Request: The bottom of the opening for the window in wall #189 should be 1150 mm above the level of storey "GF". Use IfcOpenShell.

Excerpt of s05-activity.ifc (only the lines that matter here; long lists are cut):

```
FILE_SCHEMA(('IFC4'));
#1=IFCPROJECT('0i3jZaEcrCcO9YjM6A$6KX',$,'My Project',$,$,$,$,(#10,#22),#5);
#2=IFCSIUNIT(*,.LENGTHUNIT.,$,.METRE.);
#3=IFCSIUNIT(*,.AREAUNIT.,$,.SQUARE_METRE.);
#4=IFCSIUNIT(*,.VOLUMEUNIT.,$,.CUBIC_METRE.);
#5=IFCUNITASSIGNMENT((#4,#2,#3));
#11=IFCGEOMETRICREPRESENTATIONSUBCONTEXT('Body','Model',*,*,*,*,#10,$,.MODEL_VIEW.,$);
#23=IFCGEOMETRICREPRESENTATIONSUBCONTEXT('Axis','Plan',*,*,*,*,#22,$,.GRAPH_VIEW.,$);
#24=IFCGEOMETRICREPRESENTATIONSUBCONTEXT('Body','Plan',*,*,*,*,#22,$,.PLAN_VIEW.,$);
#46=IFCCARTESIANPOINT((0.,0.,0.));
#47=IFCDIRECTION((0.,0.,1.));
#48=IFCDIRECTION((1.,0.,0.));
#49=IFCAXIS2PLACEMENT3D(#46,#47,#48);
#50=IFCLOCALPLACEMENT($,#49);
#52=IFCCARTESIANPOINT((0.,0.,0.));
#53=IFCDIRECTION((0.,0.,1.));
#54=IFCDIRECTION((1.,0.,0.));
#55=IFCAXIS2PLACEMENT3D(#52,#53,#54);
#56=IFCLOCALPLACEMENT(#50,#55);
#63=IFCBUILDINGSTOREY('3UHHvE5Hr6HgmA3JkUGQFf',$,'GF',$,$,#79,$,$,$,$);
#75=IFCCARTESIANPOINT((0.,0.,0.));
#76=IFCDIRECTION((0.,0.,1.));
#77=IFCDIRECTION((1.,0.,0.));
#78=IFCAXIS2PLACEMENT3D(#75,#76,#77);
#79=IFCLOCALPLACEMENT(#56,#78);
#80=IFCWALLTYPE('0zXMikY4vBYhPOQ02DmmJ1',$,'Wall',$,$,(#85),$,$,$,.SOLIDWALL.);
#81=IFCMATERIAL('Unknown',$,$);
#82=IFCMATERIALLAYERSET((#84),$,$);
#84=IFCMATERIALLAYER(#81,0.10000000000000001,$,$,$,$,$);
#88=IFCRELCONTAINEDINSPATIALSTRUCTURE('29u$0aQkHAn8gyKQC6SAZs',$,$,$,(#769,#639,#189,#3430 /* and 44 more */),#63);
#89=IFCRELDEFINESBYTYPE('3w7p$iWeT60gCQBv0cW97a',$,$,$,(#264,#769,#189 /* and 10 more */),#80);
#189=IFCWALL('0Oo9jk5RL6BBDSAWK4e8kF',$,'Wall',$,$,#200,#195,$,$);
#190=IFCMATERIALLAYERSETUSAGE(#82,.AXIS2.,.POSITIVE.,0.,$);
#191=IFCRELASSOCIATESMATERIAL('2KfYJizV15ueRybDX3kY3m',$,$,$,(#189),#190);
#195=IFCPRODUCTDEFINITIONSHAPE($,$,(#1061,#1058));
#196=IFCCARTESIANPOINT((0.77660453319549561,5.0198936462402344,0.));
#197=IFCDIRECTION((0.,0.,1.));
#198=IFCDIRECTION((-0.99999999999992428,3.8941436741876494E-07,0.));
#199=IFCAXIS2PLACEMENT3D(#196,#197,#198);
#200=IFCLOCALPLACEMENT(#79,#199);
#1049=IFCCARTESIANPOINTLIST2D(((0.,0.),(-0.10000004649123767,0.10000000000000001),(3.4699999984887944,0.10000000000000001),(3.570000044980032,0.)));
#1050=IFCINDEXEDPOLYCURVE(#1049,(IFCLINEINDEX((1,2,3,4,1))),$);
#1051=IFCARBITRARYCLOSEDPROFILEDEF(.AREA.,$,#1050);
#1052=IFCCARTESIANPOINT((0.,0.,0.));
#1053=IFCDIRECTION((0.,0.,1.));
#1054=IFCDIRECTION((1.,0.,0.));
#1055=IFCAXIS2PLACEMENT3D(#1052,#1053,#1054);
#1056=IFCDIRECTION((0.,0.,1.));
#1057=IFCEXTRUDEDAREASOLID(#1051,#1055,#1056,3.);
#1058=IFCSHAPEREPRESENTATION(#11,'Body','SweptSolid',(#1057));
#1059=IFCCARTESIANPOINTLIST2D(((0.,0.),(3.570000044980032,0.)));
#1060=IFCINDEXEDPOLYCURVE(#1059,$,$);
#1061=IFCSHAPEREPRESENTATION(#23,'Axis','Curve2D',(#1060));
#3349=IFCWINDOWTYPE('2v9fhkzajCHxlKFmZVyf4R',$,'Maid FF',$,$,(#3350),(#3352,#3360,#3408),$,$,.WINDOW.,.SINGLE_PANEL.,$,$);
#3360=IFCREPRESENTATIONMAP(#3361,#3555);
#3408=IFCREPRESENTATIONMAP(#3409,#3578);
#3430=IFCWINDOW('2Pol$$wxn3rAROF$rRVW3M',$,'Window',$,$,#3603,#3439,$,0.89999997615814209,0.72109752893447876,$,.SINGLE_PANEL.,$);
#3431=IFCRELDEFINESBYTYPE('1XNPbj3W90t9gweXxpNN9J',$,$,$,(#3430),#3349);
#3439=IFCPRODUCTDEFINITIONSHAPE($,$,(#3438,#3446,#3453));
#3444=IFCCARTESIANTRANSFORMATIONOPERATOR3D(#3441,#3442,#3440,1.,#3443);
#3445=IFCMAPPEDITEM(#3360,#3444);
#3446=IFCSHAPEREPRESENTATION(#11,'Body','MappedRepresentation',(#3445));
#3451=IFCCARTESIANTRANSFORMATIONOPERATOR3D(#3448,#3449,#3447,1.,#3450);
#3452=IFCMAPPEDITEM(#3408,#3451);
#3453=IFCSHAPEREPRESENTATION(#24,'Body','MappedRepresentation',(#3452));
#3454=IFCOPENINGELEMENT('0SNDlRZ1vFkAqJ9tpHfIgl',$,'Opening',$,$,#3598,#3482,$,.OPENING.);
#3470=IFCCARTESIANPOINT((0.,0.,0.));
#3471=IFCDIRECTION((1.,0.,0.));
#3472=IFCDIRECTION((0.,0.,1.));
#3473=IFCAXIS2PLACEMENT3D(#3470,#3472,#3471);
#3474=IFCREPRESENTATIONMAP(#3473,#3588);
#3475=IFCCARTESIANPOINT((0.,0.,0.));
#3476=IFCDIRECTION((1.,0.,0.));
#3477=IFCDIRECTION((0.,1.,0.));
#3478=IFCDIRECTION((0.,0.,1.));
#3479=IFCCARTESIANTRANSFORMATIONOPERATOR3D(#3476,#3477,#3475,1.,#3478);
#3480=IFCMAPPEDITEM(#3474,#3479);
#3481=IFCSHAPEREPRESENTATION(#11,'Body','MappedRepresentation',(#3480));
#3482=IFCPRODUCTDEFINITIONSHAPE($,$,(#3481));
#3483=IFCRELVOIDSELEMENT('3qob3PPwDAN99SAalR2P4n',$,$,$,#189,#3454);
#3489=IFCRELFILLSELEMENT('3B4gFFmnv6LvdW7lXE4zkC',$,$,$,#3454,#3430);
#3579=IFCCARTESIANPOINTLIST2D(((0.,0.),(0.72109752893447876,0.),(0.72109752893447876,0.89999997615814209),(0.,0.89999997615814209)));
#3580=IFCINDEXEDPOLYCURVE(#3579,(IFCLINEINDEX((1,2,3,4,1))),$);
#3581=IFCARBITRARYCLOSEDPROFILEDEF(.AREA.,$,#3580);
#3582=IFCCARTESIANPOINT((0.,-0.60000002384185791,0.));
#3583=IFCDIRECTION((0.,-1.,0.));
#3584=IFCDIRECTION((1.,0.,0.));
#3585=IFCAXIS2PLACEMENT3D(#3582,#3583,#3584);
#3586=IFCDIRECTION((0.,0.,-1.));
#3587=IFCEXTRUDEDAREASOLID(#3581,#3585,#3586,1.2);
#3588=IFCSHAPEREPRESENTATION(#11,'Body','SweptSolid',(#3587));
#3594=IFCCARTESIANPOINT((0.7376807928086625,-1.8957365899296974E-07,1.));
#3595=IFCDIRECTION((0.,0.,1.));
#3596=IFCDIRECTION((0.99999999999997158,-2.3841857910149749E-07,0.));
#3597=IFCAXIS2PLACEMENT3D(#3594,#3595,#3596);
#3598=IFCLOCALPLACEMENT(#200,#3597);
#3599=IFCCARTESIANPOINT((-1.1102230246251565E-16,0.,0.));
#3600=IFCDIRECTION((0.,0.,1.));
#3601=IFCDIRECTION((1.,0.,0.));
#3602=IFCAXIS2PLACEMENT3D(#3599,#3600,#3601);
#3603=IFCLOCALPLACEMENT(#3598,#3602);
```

```python
import numpy as np
import ifcopenshell
import ifcopenshell.api.geometry
import ifcopenshell.geom
import ifcopenshell.util.element
import ifcopenshell.util.placement
import ifcopenshell.util.shape
import ifcopenshell.util.unit

model = ifcopenshell.open("s05-activity.ifc")
unit_scale = ifcopenshell.util.unit.calculate_unit_scale(model)

window = model.by_guid("2Pol$$wxn3rAROF$rRVW3M")
opening = window.FillsVoids[0].RelatingOpeningElement
storey = ifcopenshell.util.element.get_container(window, ifc_class="IfcBuildingStorey")
level = ifcopenshell.util.placement.get_local_placement(storey.ObjectPlacement)[2, 3]

# The opening's origin need not be at the sill, so measure its lowest point.
shape = ifcopenshell.geom.create_shape(ifcopenshell.geom.settings(), opening)
bottom = ifcopenshell.util.shape.get_shape_bottom_elevation(shape, shape.geometry) / unit_scale
dz = level + 1.15 / unit_scale - bottom

shift = np.array([0.0, 0.0, dz])
# The window is placed relative to its opening, so it follows when the opening moves.
matrix = ifcopenshell.util.placement.get_local_placement(opening.ObjectPlacement)
matrix[:3, 3] += shift
ifcopenshell.api.geometry.edit_object_placement(
    model, product=opening, matrix=matrix, is_si=False, should_transform_children=True
)

print(f"moved by {dz * unit_scale:+.3f} m")

model.write("s05-activity_edited.ifc")
```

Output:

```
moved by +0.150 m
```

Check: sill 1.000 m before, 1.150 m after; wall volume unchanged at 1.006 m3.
